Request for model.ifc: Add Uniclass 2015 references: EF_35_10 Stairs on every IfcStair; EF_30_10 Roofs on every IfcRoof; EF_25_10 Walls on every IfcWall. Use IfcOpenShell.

First a look at what the model holds.

```python
import ifcopenshell

model = ifcopenshell.open("model.ifc")
print(model.schema)
print("classifications:", [c.Name for c in model.by_type("IfcClassification")])
for ifc_class in ("IfcDoor", "IfcRoof", "IfcStair", "IfcWall", "IfcWindow"):
    print(ifc_class, len(model.by_type(ifc_class)))
```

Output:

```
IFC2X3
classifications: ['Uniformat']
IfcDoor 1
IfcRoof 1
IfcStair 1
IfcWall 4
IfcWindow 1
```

```python
import ifcopenshell
import ifcopenshell.api.classification

model = ifcopenshell.open("model.ifc")

# IFC2X3 requires Source and Edition and has no link from the project to the system.
system = model.create_entity("IfcClassification", Source="NBS", Edition="2015", Name="Uniclass 2015")

codes = {
    "IfcStair": ("EF_35_10", "Stairs"),
    "IfcRoof": ("EF_30_10", "Roofs"),
    "IfcWall": ("EF_25_10", "Walls"),
}
for ifc_class, (code, name) in codes.items():
    products = model.by_type(ifc_class)
    ifcopenshell.api.classification.add_reference(
        model, products=products, classification=system, identification=code, name=name
    )
    print(code, len(products))

model.write("model-out.ifc")
```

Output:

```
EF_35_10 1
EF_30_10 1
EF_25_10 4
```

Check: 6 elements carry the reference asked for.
